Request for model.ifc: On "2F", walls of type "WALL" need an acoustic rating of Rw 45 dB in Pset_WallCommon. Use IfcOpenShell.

First a look at what the model holds.

```python
import ifcopenshell
import ifcopenshell.util.element

model = ifcopenshell.open("model.ifc")
print(model.schema)
storey = next(s for s in model.by_type("IfcBuildingStorey") if s.Name == "2F")
walls = [e for e in ifcopenshell.util.element.get_decomposition(storey) if e.is_a("IfcWall")]
seen = {}
for e in walls:
    element_type = ifcopenshell.util.element.get_type(e)
    key = (element_type.Name if element_type != e and element_type else None, ifcopenshell.util.element.get_pset(e, "Pset_WallCommon", "AcousticRating"))
    seen[key] = seen.get(key, 0) + 1
for (name, value), count in sorted(seen.items(), key=str):
    print(count, "x", name, "|", value)
```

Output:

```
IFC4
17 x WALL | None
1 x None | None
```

```python
import ifcopenshell
import ifcopenshell.api.pset
import ifcopenshell.util.element

model = ifcopenshell.open("model.ifc")

storey = next(s for s in model.by_type("IfcBuildingStorey") if s.Name == "2F")
walls = [e for e in ifcopenshell.util.element.get_decomposition(storey) if e.is_a("IfcWall")]

count = 0
for e in walls:
    element_type = ifcopenshell.util.element.get_type(e)
    if element_type in (None, e) or element_type.Name != "WALL":
        continue
    # add_pset returns the element's existing set when there is one.
    pset = ifcopenshell.api.pset.add_pset(model, product=e, name="Pset_WallCommon")
    ifcopenshell.api.pset.edit_pset(model, pset=pset, properties={"AcousticRating": "Rw 45 dB"})
    count += 1

print(count, "walls updated")

model.write("model-out.ifc")
```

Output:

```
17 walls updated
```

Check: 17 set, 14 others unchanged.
